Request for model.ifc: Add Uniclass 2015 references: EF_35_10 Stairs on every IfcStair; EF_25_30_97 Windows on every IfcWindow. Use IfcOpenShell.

First a look at what the model holds.

```python
import ifcopenshell

model = ifcopenshell.open("model.ifc")
print(model.schema)
print("classifications:", [c.Name for c in model.by_type("IfcClassification")])
for ifc_class in ("IfcDoor", "IfcRoof", "IfcStair", "IfcWall", "IfcWindow"):
    print(ifc_class, len(model.by_type(ifc_class)))
```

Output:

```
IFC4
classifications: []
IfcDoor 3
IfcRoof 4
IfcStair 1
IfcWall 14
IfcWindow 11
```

```python
import ifcopenshell
import ifcopenshell.api.classification

model = ifcopenshell.open("model.ifc")

system = ifcopenshell.api.classification.add_classification(model, classification="Uniclass 2015")

codes = {
    "IfcStair": ("EF_35_10", "Stairs"),
    "IfcWindow": ("EF_25_30_97", "Windows"),
}
for ifc_class, (code, name) in codes.items():
    products = model.by_type(ifc_class)
    ifcopenshell.api.classification.add_reference(
        model, products=products, classification=system, identification=code, name=name
    )
    print(code, len(products))

model.write("model_rev.ifc")
```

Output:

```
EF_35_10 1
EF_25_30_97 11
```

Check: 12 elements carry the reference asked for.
